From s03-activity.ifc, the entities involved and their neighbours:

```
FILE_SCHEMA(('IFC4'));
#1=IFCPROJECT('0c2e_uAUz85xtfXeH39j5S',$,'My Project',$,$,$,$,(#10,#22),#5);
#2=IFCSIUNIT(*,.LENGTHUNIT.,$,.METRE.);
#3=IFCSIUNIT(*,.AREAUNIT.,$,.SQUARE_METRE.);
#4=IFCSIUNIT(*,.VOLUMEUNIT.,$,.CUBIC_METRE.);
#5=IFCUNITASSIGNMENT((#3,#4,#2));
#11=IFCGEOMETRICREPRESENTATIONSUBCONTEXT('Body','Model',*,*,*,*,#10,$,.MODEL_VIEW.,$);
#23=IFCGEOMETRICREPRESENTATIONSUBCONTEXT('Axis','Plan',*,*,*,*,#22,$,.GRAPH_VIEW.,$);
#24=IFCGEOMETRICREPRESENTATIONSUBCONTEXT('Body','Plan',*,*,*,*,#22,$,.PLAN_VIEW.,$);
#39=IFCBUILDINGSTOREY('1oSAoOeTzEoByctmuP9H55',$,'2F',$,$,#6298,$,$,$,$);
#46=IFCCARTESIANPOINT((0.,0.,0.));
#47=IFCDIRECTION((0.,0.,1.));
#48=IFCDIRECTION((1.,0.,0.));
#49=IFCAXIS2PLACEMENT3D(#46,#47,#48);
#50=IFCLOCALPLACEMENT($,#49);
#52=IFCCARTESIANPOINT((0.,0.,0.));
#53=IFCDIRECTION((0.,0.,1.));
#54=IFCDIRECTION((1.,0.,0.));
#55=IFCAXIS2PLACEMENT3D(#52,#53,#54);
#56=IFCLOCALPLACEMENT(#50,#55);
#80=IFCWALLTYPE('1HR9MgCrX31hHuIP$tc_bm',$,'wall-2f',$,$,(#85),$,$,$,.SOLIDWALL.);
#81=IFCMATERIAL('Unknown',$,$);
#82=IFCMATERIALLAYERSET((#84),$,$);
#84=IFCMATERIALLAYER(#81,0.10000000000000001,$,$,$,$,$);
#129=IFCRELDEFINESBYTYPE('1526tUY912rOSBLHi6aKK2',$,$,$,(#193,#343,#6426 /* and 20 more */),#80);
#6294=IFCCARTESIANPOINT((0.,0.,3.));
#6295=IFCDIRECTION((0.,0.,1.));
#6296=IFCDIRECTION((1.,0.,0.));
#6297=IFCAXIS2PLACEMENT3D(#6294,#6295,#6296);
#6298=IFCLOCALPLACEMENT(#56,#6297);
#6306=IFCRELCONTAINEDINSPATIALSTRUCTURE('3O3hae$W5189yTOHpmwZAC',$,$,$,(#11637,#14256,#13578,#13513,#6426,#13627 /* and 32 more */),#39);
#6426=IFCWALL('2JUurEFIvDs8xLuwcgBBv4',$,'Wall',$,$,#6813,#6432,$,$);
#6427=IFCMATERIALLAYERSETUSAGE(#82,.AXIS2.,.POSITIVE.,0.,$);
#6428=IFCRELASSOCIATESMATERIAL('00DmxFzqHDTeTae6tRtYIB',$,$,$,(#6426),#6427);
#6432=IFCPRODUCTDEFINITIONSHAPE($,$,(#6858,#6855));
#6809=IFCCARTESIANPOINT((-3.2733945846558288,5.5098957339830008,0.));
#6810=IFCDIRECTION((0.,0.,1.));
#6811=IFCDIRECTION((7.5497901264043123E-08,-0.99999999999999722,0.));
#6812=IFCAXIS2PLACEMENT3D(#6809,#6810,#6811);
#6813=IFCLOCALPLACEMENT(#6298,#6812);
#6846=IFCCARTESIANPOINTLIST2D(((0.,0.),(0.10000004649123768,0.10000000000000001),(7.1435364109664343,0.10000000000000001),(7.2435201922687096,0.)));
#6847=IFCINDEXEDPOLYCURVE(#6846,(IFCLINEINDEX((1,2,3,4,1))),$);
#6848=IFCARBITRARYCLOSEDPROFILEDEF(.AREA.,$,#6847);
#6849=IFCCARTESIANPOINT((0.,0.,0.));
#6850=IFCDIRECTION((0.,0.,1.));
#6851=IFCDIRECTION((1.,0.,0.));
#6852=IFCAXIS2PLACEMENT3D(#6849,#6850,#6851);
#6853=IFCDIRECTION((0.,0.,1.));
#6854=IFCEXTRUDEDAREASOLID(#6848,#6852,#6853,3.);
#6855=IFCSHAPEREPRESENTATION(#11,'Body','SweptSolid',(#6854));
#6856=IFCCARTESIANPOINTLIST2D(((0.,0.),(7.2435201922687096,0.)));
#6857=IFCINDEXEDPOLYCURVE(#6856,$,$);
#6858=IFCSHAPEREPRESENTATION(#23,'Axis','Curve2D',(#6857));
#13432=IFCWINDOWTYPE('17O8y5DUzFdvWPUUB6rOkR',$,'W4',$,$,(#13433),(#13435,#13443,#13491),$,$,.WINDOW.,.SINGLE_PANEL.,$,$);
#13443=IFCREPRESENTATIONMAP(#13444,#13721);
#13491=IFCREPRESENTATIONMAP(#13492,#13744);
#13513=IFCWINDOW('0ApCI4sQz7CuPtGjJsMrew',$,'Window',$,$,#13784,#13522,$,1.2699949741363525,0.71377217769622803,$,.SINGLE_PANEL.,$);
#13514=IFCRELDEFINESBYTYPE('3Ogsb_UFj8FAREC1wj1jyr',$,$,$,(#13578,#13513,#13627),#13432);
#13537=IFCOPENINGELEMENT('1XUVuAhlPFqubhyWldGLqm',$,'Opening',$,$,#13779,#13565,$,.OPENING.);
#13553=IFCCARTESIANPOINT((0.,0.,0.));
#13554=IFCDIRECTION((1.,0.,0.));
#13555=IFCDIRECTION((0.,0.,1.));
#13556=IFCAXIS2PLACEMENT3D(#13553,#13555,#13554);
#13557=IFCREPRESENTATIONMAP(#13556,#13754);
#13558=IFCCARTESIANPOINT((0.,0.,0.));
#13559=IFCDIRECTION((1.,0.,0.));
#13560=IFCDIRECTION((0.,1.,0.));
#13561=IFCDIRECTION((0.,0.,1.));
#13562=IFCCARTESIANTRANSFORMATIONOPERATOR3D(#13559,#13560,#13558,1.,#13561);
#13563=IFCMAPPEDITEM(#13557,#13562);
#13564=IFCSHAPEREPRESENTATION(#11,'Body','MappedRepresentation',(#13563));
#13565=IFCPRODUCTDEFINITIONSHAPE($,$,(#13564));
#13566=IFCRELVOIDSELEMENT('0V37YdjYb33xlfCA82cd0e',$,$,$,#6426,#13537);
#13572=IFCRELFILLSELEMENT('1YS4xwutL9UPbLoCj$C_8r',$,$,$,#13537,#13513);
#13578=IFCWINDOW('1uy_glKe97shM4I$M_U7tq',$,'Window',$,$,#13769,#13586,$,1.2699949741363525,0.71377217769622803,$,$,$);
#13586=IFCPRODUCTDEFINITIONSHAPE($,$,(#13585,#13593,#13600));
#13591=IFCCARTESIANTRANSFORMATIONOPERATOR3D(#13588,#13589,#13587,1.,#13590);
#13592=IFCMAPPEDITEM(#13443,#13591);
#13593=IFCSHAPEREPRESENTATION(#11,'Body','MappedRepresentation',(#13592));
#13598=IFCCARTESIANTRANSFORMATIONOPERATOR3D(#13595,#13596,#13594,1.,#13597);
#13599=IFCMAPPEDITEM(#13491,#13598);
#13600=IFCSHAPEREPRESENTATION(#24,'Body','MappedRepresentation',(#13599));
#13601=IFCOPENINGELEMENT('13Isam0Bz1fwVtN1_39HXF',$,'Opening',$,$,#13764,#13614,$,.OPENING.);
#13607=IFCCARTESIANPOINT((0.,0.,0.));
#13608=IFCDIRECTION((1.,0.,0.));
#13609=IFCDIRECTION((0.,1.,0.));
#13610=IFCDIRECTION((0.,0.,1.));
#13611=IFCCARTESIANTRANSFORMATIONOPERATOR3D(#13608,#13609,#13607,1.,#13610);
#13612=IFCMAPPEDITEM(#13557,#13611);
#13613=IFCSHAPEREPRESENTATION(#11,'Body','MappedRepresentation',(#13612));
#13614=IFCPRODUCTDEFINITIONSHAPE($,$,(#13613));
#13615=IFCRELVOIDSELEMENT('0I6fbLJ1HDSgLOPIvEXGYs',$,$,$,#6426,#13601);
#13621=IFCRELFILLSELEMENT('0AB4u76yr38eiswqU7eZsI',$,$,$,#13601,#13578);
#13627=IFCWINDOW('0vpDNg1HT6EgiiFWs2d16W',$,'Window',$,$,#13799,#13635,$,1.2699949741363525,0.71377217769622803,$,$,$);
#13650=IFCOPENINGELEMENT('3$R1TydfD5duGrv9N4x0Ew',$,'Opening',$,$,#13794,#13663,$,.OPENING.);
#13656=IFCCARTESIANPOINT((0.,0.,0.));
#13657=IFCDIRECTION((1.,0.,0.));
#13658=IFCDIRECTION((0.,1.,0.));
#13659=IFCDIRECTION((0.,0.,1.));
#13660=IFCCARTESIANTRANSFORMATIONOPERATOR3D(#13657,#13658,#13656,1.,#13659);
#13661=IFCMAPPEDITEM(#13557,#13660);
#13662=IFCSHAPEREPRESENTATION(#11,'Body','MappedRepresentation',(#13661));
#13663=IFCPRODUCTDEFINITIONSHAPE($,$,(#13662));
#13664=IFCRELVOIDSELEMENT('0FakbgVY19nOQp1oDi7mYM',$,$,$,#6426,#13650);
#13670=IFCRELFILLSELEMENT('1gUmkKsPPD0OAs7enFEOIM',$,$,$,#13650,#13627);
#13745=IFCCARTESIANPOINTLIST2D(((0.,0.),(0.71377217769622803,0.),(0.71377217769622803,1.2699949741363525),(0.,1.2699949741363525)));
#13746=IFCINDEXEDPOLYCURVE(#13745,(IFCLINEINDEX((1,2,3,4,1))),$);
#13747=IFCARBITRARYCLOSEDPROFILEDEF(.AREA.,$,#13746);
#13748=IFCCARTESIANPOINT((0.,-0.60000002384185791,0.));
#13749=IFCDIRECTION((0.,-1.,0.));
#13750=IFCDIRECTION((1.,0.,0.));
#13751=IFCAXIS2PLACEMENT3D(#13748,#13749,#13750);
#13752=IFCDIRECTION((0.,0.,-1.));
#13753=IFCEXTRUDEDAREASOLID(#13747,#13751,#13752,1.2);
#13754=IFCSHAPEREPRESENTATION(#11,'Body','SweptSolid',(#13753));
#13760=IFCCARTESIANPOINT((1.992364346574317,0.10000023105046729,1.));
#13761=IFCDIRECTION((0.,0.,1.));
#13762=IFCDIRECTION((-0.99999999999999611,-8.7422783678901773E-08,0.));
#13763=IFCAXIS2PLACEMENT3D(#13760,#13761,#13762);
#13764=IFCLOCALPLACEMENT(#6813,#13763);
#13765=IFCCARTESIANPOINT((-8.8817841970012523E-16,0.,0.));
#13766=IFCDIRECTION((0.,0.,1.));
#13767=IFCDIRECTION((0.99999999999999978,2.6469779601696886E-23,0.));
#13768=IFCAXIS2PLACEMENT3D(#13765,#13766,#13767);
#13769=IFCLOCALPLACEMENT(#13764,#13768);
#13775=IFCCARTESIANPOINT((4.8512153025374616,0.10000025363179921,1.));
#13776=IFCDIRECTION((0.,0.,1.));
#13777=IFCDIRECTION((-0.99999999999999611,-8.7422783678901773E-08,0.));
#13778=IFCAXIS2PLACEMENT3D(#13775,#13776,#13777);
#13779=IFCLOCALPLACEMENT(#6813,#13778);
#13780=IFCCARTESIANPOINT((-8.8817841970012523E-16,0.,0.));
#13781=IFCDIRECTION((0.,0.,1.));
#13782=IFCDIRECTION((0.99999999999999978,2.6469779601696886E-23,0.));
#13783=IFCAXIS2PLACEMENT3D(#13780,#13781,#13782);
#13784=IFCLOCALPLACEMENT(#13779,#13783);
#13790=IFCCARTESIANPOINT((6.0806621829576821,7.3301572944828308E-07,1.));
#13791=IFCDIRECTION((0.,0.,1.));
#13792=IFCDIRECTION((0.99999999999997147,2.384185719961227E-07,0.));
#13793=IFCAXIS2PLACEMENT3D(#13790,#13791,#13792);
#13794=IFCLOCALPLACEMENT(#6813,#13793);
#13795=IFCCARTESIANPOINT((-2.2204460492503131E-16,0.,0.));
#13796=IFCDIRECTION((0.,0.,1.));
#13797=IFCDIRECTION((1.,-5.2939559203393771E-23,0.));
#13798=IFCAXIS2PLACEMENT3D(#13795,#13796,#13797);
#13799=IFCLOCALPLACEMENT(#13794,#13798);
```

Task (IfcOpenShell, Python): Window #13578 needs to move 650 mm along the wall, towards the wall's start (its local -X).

```python
import ifcopenshell
import ifcopenshell.api.geometry
import ifcopenshell.util.placement
import ifcopenshell.util.unit

model = ifcopenshell.open("s03-activity.ifc")
unit_scale = ifcopenshell.util.unit.calculate_unit_scale(model)

window = model.by_guid("1uy_glKe97shM4I$M_U7tq")
opening = window.FillsVoids[0].RelatingOpeningElement
wall = opening.VoidsElements[0].RelatingBuildingElement

wall_matrix = ifcopenshell.util.placement.get_local_placement(wall.ObjectPlacement)
shift = wall_matrix[:3, 0] * -0.65 / unit_scale
before = ifcopenshell.util.placement.get_local_placement(window.ObjectPlacement)[:3, 3].copy()

# The window is placed relative to its opening, so it follows when the opening moves.
matrix = ifcopenshell.util.placement.get_local_placement(opening.ObjectPlacement)
matrix[:3, 3] += shift
ifcopenshell.api.geometry.edit_object_placement(
    model, product=opening, matrix=matrix, is_si=False, should_transform_children=True
)

after = ifcopenshell.util.placement.get_local_placement(window.ObjectPlacement)[:3, 3]
print("window moved by", (after - before).round(3) + 0.0)

model.write("s03-activity_rev.ifc")
```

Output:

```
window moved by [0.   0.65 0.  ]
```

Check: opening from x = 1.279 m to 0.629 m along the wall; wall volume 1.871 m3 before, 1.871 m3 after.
